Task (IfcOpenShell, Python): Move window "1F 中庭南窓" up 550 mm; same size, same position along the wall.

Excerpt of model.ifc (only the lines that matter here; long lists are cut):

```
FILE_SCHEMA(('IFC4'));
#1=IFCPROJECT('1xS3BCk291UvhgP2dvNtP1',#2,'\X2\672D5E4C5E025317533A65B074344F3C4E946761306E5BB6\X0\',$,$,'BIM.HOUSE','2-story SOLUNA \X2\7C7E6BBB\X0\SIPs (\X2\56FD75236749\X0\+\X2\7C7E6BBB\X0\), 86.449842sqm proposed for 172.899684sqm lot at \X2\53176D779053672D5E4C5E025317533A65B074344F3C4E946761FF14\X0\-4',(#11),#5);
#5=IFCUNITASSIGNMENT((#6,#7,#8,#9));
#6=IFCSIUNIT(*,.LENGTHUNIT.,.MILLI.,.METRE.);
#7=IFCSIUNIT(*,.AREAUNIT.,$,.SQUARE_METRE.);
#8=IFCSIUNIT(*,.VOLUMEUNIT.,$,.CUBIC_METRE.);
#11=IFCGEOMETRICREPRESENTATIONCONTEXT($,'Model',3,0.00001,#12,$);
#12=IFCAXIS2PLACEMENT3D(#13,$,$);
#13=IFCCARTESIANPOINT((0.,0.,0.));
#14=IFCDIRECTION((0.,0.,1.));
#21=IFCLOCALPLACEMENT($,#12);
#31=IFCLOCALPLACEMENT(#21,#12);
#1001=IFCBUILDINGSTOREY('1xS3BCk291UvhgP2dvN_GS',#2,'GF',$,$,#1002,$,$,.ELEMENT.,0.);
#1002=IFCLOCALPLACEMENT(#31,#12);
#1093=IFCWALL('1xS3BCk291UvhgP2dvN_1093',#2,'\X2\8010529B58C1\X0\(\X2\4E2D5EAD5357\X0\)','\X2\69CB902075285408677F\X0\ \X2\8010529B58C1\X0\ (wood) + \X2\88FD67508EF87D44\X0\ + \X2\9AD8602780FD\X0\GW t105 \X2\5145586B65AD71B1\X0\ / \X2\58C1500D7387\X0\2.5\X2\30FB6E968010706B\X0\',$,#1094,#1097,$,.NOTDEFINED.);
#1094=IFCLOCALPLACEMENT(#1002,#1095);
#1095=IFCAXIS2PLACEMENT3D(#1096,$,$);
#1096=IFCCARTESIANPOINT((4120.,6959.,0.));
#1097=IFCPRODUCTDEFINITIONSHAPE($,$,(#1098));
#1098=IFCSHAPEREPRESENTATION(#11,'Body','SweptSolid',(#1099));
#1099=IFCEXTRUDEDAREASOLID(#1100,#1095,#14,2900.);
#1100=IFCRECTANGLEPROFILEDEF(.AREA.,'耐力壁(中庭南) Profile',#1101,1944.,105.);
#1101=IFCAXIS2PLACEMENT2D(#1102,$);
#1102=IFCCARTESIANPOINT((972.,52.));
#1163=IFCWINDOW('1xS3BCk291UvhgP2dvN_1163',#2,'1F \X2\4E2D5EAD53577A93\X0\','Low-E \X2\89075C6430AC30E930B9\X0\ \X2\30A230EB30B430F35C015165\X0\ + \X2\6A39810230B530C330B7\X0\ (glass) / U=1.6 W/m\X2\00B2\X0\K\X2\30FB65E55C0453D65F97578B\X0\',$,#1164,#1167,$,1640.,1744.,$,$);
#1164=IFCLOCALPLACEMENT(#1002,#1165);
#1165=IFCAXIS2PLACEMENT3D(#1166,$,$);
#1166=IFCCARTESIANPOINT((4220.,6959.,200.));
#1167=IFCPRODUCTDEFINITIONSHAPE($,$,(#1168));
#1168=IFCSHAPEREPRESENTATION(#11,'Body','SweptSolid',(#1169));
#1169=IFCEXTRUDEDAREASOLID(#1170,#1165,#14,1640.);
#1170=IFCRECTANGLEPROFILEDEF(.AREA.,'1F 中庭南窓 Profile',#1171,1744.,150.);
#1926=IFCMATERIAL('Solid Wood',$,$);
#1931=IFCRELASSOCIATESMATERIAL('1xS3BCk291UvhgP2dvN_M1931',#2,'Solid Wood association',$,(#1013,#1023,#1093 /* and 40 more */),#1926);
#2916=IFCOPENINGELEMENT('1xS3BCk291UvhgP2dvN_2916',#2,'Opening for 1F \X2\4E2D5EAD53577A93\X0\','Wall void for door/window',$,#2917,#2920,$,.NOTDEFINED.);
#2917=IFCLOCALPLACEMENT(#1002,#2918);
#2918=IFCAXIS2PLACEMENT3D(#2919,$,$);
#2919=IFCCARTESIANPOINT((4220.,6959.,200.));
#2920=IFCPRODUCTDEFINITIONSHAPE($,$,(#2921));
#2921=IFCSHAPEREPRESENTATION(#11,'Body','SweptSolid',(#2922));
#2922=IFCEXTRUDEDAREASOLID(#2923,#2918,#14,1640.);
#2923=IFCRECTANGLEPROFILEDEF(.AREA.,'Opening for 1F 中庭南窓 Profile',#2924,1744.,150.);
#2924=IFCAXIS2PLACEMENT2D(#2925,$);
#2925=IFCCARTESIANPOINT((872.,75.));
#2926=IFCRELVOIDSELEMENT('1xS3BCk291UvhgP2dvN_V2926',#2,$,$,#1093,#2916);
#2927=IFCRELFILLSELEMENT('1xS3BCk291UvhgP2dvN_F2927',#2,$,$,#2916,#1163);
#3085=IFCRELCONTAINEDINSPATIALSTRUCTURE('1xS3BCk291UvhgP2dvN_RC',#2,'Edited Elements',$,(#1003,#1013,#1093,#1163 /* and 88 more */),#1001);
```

```python
import numpy as np
import ifcopenshell
import ifcopenshell.api.geometry
import ifcopenshell.util.placement
import ifcopenshell.util.unit

model = ifcopenshell.open("model.ifc")
unit_scale = ifcopenshell.util.unit.calculate_unit_scale(model)

window = model.by_guid("1xS3BCk291UvhgP2dvN_1163")
opening = window.FillsVoids[0].RelatingOpeningElement
dz = 0.55 / unit_scale

shift = np.array([0.0, 0.0, dz])
# The window is not placed relative to its opening, so move both.
for product in (opening, window):
    matrix = ifcopenshell.util.placement.get_local_placement(product.ObjectPlacement)
    matrix[:3, 3] += shift
    ifcopenshell.api.geometry.edit_object_placement(model, product=product, matrix=matrix, is_si=False)

print(f"moved by {dz * unit_scale:+.3f} m")

model.write("model_edited.ifc")
```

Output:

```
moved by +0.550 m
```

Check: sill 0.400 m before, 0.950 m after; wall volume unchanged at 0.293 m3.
